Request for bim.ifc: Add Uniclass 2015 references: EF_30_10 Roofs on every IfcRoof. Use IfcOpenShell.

First a look at what the model holds.

```python
import ifcopenshell

model = ifcopenshell.open("bim.ifc")
print(model.schema)
print("classifications:", [c.Name for c in model.by_type("IfcClassification")])
for ifc_class in ("IfcDoor", "IfcRoof", "IfcStair", "IfcWall", "IfcWindow"):
    print(ifc_class, len(model.by_type(ifc_class)))
```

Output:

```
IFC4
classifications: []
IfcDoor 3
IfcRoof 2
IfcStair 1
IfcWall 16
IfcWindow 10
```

```python
import ifcopenshell
import ifcopenshell.api.classification

model = ifcopenshell.open("bim.ifc")

system = ifcopenshell.api.classification.add_classification(model, classification="Uniclass 2015")

codes = {
    "IfcRoof": ("EF_30_10", "Roofs"),
}
for ifc_class, (code, name) in codes.items():
    products = model.by_type(ifc_class)
    ifcopenshell.api.classification.add_reference(
        model, products=products, classification=system, identification=code, name=name
    )
    print(code, len(products))

model.write("bim_edited.ifc")
```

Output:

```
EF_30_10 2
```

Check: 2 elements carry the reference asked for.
